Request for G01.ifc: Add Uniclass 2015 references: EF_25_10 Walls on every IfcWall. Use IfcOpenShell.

First a look at what the model holds.

```python
import ifcopenshell

model = ifcopenshell.open("G01.ifc")
print(model.schema)
print("classifications:", [c.Name for c in model.by_type("IfcClassification")])
for ifc_class in ("IfcDoor", "IfcRoof", "IfcStair", "IfcWall", "IfcWindow"):
    print(ifc_class, len(model.by_type(ifc_class)))
```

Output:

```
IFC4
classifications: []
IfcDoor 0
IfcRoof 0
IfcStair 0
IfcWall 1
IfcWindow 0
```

```python
import ifcopenshell
import ifcopenshell.api.classification

model = ifcopenshell.open("G01.ifc")

system = ifcopenshell.api.classification.add_classification(model, classification="Uniclass 2015")

codes = {
    "IfcWall": ("EF_25_10", "Walls"),
}
for ifc_class, (code, name) in codes.items():
    products = model.by_type(ifc_class)
    ifcopenshell.api.classification.add_reference(
        model, products=products, classification=system, identification=code, name=name
    )
    print(code, len(products))

model.write("G01_rev.ifc")
```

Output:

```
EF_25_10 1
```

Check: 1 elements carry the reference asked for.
